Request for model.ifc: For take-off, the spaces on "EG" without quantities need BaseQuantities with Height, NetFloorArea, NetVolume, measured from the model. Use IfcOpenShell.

First a look at what the model holds.

```python
import ifcopenshell
import ifcopenshell.util.element
import ifcopenshell.util.unit

model = ifcopenshell.open("model.ifc")
print(model.schema)
for unit_type in ("LENGTHUNIT", "AREAUNIT", "VOLUMEUNIT"):
    print(unit_type, ifcopenshell.util.unit.calculate_unit_scale(model, unit_type))
storey = next(s for s in model.by_type("IfcBuildingStorey") if s.Name == "EG")
spaces = [e for e in ifcopenshell.util.element.get_decomposition(storey) if e.is_a("IfcSpace")]
for e in sorted(spaces, key=lambda e: e.id()):
    print(e.id(), e.is_a(), e.Name, list(ifcopenshell.util.element.get_psets(e, qtos_only=True)), sep=" | ")
```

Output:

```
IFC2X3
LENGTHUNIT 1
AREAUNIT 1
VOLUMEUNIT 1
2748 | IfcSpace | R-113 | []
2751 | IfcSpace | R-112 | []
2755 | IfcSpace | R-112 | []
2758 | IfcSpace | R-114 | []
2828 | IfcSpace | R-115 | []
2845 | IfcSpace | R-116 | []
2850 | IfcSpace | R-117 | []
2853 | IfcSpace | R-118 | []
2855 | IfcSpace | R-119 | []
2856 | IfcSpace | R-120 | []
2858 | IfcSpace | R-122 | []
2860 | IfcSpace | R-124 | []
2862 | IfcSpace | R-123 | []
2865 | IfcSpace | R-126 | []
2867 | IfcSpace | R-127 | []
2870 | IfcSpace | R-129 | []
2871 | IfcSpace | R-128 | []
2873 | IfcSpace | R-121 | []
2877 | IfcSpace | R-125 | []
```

```python
import ifcopenshell
import ifcopenshell.api.pset
import ifcopenshell.geom
import ifcopenshell.util.element
import ifcopenshell.util.shape
import ifcopenshell.util.unit

model = ifcopenshell.open("model.ifc")
unit_scale = ifcopenshell.util.unit.calculate_unit_scale(model)
area_scale = ifcopenshell.util.unit.calculate_unit_scale(model, "AREAUNIT")
volume_scale = ifcopenshell.util.unit.calculate_unit_scale(model, "VOLUMEUNIT")
settings = ifcopenshell.geom.settings()

storey = next(s for s in model.by_type("IfcBuildingStorey") if s.Name == "EG")
spaces = [e for e in ifcopenshell.util.element.get_decomposition(storey) if e.is_a("IfcSpace")]

for e in sorted(spaces, key=lambda e: e.id()):
    if ifcopenshell.util.element.get_psets(e, qtos_only=True, should_inherit=False):
        continue
    # Geometry comes back in metres, in the element's own axes.
    shape = ifcopenshell.geom.create_shape(settings, e)
    values = {
        "Height": ifcopenshell.util.shape.get_z(shape.geometry) / unit_scale,
        "NetFloorArea": ifcopenshell.util.shape.get_footprint_area(shape.geometry) / area_scale,
        "NetVolume": ifcopenshell.util.shape.get_volume(shape.geometry) / volume_scale,
    }
    qto = ifcopenshell.api.pset.add_qto(model, product=e, name="BaseQuantities")
    ifcopenshell.api.pset.edit_qto(model, qto=qto, properties=values)
    print(e.id(), {k: round(v, 3) for k, v in values.items()})

model.write("model_rev.ifc")
```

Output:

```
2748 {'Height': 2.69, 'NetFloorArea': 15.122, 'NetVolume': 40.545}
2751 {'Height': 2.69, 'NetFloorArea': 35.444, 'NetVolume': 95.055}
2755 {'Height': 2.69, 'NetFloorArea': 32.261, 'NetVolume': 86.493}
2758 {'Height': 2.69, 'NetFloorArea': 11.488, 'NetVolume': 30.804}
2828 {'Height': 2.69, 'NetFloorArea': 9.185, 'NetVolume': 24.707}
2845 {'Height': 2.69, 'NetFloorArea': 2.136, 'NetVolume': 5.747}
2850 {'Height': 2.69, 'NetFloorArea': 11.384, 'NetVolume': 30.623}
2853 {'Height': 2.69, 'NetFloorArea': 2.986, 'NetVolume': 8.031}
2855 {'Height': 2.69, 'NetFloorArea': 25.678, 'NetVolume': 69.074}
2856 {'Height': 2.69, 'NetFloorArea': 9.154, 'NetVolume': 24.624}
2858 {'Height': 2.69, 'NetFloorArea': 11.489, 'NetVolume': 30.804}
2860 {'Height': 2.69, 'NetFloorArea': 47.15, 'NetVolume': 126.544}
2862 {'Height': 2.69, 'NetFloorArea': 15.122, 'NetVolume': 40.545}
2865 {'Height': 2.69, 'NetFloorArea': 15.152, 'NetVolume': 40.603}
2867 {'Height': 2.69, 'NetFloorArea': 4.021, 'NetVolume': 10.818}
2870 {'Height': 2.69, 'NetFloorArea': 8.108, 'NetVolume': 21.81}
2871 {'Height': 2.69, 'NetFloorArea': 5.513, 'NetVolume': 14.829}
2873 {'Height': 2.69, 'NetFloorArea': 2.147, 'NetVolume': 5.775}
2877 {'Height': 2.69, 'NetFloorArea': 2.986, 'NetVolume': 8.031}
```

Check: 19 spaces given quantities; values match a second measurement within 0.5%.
